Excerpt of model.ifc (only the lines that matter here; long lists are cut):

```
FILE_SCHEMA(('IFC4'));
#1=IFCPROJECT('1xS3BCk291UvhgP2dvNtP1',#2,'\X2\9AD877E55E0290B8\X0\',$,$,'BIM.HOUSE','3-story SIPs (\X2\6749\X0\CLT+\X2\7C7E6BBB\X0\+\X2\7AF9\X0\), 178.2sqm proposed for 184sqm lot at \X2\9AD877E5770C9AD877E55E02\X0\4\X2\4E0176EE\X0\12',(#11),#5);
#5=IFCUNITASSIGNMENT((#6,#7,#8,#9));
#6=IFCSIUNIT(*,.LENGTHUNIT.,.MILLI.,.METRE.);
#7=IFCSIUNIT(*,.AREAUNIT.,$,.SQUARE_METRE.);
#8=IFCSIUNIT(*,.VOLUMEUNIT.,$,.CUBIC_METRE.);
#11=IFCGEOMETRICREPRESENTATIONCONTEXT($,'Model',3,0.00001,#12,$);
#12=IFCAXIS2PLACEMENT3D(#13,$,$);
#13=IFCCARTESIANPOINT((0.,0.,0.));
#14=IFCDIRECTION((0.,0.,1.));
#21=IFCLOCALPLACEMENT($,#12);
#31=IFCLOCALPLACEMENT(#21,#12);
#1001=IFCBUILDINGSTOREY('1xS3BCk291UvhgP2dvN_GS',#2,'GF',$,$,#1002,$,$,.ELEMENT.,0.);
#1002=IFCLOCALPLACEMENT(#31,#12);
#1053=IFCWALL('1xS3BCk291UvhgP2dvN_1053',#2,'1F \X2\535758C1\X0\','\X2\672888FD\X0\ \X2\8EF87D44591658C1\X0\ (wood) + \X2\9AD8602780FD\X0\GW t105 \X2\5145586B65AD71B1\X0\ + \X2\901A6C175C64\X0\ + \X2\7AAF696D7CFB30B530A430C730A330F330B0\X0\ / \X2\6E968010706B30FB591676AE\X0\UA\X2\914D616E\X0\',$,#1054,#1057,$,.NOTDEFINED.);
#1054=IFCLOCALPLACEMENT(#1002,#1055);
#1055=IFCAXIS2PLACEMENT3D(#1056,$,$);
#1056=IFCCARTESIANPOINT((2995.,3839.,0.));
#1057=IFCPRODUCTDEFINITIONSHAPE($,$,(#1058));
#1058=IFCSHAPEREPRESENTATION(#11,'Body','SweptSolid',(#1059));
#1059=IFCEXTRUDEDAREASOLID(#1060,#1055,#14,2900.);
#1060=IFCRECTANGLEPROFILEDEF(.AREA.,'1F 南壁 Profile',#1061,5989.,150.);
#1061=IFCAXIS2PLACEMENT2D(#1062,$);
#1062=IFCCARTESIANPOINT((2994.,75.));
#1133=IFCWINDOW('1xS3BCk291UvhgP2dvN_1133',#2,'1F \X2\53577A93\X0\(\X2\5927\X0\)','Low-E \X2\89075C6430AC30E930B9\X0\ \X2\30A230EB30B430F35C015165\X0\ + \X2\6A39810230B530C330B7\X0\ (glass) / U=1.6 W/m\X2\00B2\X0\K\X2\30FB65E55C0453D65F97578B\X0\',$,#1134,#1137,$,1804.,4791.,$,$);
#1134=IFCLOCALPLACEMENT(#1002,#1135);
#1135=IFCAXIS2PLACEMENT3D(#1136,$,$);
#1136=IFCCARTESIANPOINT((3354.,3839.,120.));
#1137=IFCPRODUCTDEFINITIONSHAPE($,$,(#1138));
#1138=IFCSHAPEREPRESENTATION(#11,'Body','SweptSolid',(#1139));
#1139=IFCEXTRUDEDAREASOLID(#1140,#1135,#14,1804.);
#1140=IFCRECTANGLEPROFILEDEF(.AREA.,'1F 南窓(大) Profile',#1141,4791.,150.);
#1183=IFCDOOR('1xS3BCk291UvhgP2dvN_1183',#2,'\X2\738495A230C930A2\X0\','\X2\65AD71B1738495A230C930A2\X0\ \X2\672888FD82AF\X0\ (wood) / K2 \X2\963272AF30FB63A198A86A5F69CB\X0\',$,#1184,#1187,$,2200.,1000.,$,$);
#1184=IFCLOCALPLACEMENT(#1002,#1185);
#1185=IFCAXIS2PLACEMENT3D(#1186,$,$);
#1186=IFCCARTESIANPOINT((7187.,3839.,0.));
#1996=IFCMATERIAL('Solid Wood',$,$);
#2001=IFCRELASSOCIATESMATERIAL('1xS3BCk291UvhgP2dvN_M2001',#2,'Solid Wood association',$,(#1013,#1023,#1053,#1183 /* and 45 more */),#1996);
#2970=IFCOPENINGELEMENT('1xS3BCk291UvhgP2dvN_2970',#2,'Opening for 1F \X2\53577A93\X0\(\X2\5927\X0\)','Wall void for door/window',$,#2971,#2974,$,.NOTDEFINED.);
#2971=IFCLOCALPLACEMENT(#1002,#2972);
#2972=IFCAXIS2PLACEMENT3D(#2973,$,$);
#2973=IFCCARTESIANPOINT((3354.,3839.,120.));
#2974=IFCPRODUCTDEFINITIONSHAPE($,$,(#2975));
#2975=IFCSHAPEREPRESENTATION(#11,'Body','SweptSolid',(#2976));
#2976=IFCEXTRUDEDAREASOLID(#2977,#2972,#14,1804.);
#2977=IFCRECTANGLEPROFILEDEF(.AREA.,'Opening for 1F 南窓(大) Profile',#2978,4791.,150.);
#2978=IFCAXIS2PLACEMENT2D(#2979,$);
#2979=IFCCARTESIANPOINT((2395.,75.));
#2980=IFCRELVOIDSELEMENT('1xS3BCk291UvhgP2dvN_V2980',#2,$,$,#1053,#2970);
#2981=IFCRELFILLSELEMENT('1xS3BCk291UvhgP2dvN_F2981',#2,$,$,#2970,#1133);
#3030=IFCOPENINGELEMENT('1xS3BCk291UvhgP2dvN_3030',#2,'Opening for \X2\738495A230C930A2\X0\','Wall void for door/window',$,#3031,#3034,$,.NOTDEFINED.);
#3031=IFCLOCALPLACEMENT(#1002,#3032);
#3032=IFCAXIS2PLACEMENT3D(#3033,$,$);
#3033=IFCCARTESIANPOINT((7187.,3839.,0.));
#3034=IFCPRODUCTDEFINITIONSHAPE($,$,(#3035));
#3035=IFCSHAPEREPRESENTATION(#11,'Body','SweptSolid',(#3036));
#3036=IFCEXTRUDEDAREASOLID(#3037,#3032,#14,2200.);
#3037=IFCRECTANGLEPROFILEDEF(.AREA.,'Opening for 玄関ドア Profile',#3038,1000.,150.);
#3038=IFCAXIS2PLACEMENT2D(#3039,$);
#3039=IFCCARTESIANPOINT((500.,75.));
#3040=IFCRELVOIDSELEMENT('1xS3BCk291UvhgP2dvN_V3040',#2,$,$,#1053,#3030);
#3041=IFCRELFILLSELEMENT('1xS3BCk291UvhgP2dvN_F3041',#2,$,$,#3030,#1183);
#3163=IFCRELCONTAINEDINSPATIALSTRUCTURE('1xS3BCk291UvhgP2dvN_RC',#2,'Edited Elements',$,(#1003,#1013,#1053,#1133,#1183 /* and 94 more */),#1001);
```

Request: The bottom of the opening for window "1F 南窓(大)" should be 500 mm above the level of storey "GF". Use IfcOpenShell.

```python
import numpy as np
import ifcopenshell
import ifcopenshell.api.geometry
import ifcopenshell.geom
import ifcopenshell.util.element
import ifcopenshell.util.placement
import ifcopenshell.util.shape
import ifcopenshell.util.unit

model = ifcopenshell.open("model.ifc")
unit_scale = ifcopenshell.util.unit.calculate_unit_scale(model)

window = model.by_guid("1xS3BCk291UvhgP2dvN_1133")
opening = window.FillsVoids[0].RelatingOpeningElement
storey = ifcopenshell.util.element.get_container(window, ifc_class="IfcBuildingStorey")
level = ifcopenshell.util.placement.get_local_placement(storey.ObjectPlacement)[2, 3]

# The opening's origin need not be at the sill, so measure its lowest point.
shape = ifcopenshell.geom.create_shape(ifcopenshell.geom.settings(), opening)
bottom = ifcopenshell.util.shape.get_shape_bottom_elevation(shape, shape.geometry) / unit_scale
dz = level + 500.0 - bottom

shift = np.array([0.0, 0.0, dz])
# The window is not placed relative to its opening, so move both.
for product in (opening, window):
    matrix = ifcopenshell.util.placement.get_local_placement(product.ObjectPlacement)
    matrix[:3, 3] += shift
    ifcopenshell.api.geometry.edit_object_placement(model, product=product, matrix=matrix, is_si=False)

print(f"moved by {dz * unit_scale:+.3f} m")

model.write("model_rev.ifc")
```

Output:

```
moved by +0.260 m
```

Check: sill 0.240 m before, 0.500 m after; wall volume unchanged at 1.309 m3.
